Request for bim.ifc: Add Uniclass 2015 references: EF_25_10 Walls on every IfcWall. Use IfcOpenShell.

First a look at what the model holds.

```python
import ifcopenshell

model = ifcopenshell.open("bim.ifc")
print(model.schema)
print("classifications:", [c.Name for c in model.by_type("IfcClassification")])
for ifc_class in ("IfcDoor", "IfcRoof", "IfcStair", "IfcWall", "IfcWindow"):
    print(ifc_class, len(model.by_type(ifc_class)))
```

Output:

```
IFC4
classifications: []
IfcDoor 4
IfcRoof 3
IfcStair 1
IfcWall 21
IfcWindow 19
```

```python
import ifcopenshell
import ifcopenshell.api.classification

model = ifcopenshell.open("bim.ifc")

system = ifcopenshell.api.classification.add_classification(model, classification="Uniclass 2015")

codes = {
    "IfcWall": ("EF_25_10", "Walls"),
}
for ifc_class, (code, name) in codes.items():
    products = model.by_type(ifc_class)
    ifcopenshell.api.classification.add_reference(
        model, products=products, classification=system, identification=code, name=name
    )
    print(code, len(products))

model.write("bim-out.ifc")
```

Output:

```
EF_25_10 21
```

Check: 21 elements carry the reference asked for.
